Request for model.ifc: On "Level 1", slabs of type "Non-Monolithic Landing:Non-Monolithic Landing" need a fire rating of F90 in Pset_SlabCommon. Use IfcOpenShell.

First a look at what the model holds.

```python
import ifcopenshell
import ifcopenshell.util.element

model = ifcopenshell.open("model.ifc")
print(model.schema)
storey = next(s for s in model.by_type("IfcBuildingStorey") if s.Name == "Level 1")
slabs = [e for e in ifcopenshell.util.element.get_decomposition(storey) if e.is_a("IfcSlab")]
seen = {}
for e in slabs:
    element_type = ifcopenshell.util.element.get_type(e)
    key = (element_type.Name if element_type != e and element_type else None, ifcopenshell.util.element.get_pset(e, "Pset_SlabCommon", "FireRating"))
    seen[key] = seen.get(key, 0) + 1
for (name, value), count in sorted(seen.items(), key=str):
    print(count, "x", name, "|", value)
```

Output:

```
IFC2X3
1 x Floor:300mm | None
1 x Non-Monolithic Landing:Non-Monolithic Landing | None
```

```python
import ifcopenshell
import ifcopenshell.api.pset
import ifcopenshell.util.element

model = ifcopenshell.open("model.ifc")

storey = next(s for s in model.by_type("IfcBuildingStorey") if s.Name == "Level 1")
slabs = [e for e in ifcopenshell.util.element.get_decomposition(storey) if e.is_a("IfcSlab")]

count = 0
for e in slabs:
    element_type = ifcopenshell.util.element.get_type(e)
    if element_type in (None, e) or element_type.Name != "Non-Monolithic Landing:Non-Monolithic Landing":
        continue
    # add_pset returns the element's existing set when there is one.
    pset = ifcopenshell.api.pset.add_pset(model, product=e, name="Pset_SlabCommon")
    ifcopenshell.api.pset.edit_pset(model, pset=pset, properties={"FireRating": "F90"})
    count += 1

print(count, "slabs updated")

model.write("model_rev.ifc")
```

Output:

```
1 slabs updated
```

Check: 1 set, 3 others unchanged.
